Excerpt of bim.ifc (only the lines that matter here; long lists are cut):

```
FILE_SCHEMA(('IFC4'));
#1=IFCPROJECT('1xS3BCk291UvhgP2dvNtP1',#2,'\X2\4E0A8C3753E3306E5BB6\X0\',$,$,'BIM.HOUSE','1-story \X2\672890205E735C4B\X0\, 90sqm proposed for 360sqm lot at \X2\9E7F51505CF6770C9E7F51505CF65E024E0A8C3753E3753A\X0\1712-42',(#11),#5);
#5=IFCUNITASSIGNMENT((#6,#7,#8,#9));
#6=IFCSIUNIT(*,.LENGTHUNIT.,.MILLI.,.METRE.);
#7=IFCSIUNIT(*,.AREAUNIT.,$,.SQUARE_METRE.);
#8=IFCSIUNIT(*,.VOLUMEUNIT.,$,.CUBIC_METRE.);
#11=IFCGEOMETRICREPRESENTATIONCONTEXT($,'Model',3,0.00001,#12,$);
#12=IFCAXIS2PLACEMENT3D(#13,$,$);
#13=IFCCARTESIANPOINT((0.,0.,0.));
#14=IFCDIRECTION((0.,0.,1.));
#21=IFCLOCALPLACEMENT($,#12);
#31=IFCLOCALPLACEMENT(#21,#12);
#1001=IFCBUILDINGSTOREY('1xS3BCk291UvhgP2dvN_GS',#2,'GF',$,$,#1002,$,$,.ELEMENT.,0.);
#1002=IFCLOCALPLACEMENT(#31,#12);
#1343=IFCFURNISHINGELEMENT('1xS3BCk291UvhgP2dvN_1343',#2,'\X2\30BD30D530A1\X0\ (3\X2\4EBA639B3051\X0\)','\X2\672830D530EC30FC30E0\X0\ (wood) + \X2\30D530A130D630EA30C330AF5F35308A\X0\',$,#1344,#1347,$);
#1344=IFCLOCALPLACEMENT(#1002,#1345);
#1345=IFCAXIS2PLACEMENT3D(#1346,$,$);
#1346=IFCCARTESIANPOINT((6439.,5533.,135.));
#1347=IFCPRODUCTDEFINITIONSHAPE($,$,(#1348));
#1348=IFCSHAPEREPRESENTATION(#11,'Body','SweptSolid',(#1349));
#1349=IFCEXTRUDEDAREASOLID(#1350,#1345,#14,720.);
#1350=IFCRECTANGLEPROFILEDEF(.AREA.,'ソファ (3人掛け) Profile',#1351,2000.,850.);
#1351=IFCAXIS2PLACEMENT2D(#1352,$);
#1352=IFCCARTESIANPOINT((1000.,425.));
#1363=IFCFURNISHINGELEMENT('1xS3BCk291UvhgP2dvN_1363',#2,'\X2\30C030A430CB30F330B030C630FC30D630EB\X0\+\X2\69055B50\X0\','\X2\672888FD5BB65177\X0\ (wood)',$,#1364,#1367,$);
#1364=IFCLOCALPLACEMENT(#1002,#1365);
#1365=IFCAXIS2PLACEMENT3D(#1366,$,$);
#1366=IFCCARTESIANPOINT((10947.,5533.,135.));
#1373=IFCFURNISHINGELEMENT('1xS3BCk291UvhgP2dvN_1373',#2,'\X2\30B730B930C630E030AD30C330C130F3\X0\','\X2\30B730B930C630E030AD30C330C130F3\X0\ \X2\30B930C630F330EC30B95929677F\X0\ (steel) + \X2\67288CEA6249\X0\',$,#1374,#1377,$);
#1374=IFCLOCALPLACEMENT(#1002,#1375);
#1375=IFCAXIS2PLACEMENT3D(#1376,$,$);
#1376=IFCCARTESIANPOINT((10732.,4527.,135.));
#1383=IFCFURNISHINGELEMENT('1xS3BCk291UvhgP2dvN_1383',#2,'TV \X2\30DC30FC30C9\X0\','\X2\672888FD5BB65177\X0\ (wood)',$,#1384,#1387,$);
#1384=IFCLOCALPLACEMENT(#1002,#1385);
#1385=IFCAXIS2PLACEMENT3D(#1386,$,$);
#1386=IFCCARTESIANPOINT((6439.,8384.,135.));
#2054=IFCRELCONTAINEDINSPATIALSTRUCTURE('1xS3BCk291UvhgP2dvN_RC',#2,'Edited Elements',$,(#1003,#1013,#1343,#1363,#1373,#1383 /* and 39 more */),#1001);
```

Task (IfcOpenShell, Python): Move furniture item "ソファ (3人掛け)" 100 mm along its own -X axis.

```python
import ifcopenshell
import ifcopenshell.api.geometry
import ifcopenshell.util.placement

model = ifcopenshell.open("bim.ifc")

item = model.by_guid("1xS3BCk291UvhgP2dvN_1343")
matrix = ifcopenshell.util.placement.get_local_placement(item.ObjectPlacement)
matrix[:3, 3] -= matrix[:3, 0] * 100.0
ifcopenshell.api.geometry.edit_object_placement(model, product=item, matrix=matrix, is_si=False)

print(ifcopenshell.util.placement.get_local_placement(item.ObjectPlacement).round(3) + 0.0)

model.write("bim_v2.ifc")
```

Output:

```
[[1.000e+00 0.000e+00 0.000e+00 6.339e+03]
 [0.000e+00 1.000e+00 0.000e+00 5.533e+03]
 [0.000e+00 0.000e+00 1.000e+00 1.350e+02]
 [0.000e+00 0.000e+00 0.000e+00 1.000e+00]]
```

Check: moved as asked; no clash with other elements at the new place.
